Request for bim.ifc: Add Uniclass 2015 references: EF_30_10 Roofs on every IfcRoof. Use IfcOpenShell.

First a look at what the model holds.

```python
import ifcopenshell

model = ifcopenshell.open("bim.ifc")
print(model.schema)
print("classifications:", [c.Name for c in model.by_type("IfcClassification")])
for ifc_class in ("IfcDoor", "IfcRoof", "IfcStair", "IfcWall", "IfcWindow"):
    print(ifc_class, len(model.by_type(ifc_class)))
```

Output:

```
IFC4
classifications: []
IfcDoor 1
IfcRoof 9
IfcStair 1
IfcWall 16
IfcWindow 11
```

```python
import ifcopenshell
import ifcopenshell.api.classification

model = ifcopenshell.open("bim.ifc")

system = ifcopenshell.api.classification.add_classification(model, classification="Uniclass 2015")

codes = {
    "IfcRoof": ("EF_30_10", "Roofs"),
}
for ifc_class, (code, name) in codes.items():
    products = model.by_type(ifc_class)
    ifcopenshell.api.classification.add_reference(
        model, products=products, classification=system, identification=code, name=name
    )
    print(code, len(products))

model.write("bim_v2.ifc")
```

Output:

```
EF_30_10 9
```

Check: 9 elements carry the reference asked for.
